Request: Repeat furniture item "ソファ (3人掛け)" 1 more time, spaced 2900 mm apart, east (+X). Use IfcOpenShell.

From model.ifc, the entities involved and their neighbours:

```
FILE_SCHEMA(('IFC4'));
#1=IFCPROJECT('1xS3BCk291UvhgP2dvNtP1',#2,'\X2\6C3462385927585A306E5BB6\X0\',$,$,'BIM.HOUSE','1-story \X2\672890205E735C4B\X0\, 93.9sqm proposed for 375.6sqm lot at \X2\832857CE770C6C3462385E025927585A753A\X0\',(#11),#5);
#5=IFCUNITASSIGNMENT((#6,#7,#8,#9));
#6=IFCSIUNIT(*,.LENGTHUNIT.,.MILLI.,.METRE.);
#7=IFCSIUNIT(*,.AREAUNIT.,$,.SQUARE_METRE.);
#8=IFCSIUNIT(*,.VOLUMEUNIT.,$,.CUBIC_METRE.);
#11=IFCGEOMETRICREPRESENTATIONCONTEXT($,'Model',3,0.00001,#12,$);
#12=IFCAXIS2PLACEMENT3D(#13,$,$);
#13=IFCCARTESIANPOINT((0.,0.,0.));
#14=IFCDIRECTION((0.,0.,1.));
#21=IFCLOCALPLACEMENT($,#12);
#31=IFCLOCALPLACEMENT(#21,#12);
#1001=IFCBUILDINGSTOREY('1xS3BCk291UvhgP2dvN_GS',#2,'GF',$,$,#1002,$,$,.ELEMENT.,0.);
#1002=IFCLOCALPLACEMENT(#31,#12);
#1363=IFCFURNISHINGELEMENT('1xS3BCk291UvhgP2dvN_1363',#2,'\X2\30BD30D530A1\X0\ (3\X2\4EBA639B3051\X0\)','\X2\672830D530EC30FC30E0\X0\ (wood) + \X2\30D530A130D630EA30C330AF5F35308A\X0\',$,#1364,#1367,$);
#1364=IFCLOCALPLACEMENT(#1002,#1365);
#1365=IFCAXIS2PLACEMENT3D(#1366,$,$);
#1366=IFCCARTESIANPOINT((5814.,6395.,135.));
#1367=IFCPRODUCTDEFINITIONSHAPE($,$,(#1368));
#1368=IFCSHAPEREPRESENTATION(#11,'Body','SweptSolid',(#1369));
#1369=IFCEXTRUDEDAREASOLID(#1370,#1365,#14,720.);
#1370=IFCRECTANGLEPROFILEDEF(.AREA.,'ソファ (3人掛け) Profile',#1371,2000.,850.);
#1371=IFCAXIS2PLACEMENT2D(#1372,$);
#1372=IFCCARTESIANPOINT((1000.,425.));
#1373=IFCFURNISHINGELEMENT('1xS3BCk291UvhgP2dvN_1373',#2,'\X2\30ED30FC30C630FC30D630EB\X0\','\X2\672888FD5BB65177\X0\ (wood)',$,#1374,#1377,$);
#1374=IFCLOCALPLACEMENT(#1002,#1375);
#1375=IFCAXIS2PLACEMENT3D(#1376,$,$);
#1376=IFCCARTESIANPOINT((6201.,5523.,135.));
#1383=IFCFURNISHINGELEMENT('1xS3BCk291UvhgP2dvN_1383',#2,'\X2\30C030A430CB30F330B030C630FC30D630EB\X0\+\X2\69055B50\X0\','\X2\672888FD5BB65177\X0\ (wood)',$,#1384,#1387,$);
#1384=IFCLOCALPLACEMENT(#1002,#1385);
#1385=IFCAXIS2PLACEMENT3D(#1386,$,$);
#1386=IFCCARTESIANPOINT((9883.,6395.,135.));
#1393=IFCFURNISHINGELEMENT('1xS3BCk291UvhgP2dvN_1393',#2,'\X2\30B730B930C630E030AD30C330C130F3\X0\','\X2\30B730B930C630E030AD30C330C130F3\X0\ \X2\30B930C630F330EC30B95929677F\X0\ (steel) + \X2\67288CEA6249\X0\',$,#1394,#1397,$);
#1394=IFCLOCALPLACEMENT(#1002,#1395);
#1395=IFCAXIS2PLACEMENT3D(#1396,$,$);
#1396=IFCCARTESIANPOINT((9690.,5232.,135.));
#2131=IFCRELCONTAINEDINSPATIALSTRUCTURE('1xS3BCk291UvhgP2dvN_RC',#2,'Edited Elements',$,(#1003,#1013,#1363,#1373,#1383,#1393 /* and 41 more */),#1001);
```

```python
import numpy as np
import ifcopenshell
import ifcopenshell.api.geometry
import ifcopenshell.api.root
import ifcopenshell.util.element
import ifcopenshell.util.placement
import ifcopenshell.util.unit

model = ifcopenshell.open("model.ifc")
unit_scale = ifcopenshell.util.unit.calculate_unit_scale(model)


def reuse_history(source, copy):
    """copy_class also copies each property set's owner history, people and application; keep the originals."""
    for rel in copy.IsDefinedBy:
        if rel.is_a("IfcRelDefinesByProperties") and (history := rel.RelatingPropertyDefinition.OwnerHistory):
            rel.RelatingPropertyDefinition.OwnerHistory = source.OwnerHistory
            ifcopenshell.util.element.remove_deep2(model, history)


source = model.by_id(1363)
base = ifcopenshell.util.placement.get_local_placement(source.ObjectPlacement)
step = np.array([1.0, 0.0, 0.0]) * 2.9 / unit_scale

for i in range(1, 2):
    copy = ifcopenshell.api.root.copy_class(model, product=source)
    copy.Representation = ifcopenshell.util.element.copy_deep(
        model, source.Representation, exclude=["IfcGeometricRepresentationContext", "IfcRepresentationMap"]
    )
    reuse_history(source, copy)
    matrix = base.copy()
    matrix[:3, 3] += i * step
    print("added at", matrix[:3, 3].round(3) + 0.0)
    ifcopenshell.api.geometry.edit_object_placement(model, product=copy, matrix=matrix, is_si=False)

model.write("model_edited.ifc")
```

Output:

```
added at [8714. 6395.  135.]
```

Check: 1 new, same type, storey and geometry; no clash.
